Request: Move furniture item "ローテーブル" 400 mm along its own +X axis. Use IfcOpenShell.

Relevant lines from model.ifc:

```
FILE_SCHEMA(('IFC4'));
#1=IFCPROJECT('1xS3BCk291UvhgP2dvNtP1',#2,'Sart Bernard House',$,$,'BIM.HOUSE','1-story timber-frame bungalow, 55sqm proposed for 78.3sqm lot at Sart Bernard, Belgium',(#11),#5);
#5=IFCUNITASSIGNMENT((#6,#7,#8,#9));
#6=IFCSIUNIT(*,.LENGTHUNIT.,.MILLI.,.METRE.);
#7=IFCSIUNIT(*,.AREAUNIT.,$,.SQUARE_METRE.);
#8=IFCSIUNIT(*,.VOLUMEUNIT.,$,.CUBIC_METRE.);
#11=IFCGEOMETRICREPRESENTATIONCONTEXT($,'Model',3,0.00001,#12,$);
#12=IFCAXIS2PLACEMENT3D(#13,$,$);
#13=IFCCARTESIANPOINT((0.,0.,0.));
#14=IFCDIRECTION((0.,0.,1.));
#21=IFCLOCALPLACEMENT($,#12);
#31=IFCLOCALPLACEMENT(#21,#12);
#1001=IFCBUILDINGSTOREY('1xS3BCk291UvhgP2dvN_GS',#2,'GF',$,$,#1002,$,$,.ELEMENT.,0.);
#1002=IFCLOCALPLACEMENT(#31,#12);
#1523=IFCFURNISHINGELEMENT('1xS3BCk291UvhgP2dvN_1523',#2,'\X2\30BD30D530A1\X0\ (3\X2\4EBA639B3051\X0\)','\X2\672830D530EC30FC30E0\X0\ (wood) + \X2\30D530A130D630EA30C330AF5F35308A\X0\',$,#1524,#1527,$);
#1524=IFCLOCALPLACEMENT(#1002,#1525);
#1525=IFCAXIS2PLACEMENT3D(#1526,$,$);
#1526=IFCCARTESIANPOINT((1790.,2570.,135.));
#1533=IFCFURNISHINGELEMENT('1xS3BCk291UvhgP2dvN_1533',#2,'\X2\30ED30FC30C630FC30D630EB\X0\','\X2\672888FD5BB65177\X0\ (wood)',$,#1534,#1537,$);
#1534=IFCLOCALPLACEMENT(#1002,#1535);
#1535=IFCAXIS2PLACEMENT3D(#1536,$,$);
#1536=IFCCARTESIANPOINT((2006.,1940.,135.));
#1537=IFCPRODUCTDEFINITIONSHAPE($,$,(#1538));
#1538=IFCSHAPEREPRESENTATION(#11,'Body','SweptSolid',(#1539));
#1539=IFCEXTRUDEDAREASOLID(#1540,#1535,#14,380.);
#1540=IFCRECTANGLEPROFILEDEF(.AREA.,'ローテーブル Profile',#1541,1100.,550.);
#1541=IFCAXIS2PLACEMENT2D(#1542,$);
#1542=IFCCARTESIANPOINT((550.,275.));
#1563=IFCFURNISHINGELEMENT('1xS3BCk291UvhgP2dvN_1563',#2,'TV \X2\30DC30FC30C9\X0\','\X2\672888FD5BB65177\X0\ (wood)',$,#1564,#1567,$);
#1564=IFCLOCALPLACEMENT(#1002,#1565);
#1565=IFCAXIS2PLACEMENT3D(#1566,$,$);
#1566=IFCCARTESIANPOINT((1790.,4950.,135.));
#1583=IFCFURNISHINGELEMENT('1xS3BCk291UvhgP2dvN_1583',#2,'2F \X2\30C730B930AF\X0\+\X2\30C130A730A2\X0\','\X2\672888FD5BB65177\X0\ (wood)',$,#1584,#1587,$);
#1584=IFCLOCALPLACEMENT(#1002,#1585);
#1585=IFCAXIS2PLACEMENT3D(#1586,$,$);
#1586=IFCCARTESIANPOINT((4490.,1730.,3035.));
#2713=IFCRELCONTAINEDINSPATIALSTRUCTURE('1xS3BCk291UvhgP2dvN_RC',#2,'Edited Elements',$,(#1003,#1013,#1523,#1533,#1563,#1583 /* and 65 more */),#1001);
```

```python
import ifcopenshell
import ifcopenshell.api.geometry
import ifcopenshell.util.placement
import ifcopenshell.util.unit

model = ifcopenshell.open("model.ifc")
unit_scale = ifcopenshell.util.unit.calculate_unit_scale(model)

item = model.by_guid("1xS3BCk291UvhgP2dvN_1533")
matrix = ifcopenshell.util.placement.get_local_placement(item.ObjectPlacement)
matrix[:3, 3] += matrix[:3, 0] * 0.4 / unit_scale
ifcopenshell.api.geometry.edit_object_placement(model, product=item, matrix=matrix, is_si=False)

print(ifcopenshell.util.placement.get_local_placement(item.ObjectPlacement).round(3) + 0.0)

model.write("model_v2.ifc")
```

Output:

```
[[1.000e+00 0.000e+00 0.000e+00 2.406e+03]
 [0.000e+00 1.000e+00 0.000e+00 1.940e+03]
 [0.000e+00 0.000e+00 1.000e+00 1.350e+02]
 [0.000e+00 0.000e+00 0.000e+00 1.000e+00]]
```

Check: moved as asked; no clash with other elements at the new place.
